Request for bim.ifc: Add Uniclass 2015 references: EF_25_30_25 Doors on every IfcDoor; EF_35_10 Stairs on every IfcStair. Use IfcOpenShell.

First a look at what the model holds.

```python
import ifcopenshell

model = ifcopenshell.open("bim.ifc")
print(model.schema)
print("classifications:", [c.Name for c in model.by_type("IfcClassification")])
for ifc_class in ("IfcDoor", "IfcRoof", "IfcStair", "IfcWall", "IfcWindow"):
    print(ifc_class, len(model.by_type(ifc_class)))
```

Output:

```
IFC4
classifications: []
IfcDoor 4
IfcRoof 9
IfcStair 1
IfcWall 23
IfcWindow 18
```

```python
import ifcopenshell
import ifcopenshell.api.classification

model = ifcopenshell.open("bim.ifc")

system = ifcopenshell.api.classification.add_classification(model, classification="Uniclass 2015")

codes = {
    "IfcDoor": ("EF_25_30_25", "Doors"),
    "IfcStair": ("EF_35_10", "Stairs"),
}
for ifc_class, (code, name) in codes.items():
    products = model.by_type(ifc_class)
    ifcopenshell.api.classification.add_reference(
        model, products=products, classification=system, identification=code, name=name
    )
    print(code, len(products))

model.write("bim_updated.ifc")
```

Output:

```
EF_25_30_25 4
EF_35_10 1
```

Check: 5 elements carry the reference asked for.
